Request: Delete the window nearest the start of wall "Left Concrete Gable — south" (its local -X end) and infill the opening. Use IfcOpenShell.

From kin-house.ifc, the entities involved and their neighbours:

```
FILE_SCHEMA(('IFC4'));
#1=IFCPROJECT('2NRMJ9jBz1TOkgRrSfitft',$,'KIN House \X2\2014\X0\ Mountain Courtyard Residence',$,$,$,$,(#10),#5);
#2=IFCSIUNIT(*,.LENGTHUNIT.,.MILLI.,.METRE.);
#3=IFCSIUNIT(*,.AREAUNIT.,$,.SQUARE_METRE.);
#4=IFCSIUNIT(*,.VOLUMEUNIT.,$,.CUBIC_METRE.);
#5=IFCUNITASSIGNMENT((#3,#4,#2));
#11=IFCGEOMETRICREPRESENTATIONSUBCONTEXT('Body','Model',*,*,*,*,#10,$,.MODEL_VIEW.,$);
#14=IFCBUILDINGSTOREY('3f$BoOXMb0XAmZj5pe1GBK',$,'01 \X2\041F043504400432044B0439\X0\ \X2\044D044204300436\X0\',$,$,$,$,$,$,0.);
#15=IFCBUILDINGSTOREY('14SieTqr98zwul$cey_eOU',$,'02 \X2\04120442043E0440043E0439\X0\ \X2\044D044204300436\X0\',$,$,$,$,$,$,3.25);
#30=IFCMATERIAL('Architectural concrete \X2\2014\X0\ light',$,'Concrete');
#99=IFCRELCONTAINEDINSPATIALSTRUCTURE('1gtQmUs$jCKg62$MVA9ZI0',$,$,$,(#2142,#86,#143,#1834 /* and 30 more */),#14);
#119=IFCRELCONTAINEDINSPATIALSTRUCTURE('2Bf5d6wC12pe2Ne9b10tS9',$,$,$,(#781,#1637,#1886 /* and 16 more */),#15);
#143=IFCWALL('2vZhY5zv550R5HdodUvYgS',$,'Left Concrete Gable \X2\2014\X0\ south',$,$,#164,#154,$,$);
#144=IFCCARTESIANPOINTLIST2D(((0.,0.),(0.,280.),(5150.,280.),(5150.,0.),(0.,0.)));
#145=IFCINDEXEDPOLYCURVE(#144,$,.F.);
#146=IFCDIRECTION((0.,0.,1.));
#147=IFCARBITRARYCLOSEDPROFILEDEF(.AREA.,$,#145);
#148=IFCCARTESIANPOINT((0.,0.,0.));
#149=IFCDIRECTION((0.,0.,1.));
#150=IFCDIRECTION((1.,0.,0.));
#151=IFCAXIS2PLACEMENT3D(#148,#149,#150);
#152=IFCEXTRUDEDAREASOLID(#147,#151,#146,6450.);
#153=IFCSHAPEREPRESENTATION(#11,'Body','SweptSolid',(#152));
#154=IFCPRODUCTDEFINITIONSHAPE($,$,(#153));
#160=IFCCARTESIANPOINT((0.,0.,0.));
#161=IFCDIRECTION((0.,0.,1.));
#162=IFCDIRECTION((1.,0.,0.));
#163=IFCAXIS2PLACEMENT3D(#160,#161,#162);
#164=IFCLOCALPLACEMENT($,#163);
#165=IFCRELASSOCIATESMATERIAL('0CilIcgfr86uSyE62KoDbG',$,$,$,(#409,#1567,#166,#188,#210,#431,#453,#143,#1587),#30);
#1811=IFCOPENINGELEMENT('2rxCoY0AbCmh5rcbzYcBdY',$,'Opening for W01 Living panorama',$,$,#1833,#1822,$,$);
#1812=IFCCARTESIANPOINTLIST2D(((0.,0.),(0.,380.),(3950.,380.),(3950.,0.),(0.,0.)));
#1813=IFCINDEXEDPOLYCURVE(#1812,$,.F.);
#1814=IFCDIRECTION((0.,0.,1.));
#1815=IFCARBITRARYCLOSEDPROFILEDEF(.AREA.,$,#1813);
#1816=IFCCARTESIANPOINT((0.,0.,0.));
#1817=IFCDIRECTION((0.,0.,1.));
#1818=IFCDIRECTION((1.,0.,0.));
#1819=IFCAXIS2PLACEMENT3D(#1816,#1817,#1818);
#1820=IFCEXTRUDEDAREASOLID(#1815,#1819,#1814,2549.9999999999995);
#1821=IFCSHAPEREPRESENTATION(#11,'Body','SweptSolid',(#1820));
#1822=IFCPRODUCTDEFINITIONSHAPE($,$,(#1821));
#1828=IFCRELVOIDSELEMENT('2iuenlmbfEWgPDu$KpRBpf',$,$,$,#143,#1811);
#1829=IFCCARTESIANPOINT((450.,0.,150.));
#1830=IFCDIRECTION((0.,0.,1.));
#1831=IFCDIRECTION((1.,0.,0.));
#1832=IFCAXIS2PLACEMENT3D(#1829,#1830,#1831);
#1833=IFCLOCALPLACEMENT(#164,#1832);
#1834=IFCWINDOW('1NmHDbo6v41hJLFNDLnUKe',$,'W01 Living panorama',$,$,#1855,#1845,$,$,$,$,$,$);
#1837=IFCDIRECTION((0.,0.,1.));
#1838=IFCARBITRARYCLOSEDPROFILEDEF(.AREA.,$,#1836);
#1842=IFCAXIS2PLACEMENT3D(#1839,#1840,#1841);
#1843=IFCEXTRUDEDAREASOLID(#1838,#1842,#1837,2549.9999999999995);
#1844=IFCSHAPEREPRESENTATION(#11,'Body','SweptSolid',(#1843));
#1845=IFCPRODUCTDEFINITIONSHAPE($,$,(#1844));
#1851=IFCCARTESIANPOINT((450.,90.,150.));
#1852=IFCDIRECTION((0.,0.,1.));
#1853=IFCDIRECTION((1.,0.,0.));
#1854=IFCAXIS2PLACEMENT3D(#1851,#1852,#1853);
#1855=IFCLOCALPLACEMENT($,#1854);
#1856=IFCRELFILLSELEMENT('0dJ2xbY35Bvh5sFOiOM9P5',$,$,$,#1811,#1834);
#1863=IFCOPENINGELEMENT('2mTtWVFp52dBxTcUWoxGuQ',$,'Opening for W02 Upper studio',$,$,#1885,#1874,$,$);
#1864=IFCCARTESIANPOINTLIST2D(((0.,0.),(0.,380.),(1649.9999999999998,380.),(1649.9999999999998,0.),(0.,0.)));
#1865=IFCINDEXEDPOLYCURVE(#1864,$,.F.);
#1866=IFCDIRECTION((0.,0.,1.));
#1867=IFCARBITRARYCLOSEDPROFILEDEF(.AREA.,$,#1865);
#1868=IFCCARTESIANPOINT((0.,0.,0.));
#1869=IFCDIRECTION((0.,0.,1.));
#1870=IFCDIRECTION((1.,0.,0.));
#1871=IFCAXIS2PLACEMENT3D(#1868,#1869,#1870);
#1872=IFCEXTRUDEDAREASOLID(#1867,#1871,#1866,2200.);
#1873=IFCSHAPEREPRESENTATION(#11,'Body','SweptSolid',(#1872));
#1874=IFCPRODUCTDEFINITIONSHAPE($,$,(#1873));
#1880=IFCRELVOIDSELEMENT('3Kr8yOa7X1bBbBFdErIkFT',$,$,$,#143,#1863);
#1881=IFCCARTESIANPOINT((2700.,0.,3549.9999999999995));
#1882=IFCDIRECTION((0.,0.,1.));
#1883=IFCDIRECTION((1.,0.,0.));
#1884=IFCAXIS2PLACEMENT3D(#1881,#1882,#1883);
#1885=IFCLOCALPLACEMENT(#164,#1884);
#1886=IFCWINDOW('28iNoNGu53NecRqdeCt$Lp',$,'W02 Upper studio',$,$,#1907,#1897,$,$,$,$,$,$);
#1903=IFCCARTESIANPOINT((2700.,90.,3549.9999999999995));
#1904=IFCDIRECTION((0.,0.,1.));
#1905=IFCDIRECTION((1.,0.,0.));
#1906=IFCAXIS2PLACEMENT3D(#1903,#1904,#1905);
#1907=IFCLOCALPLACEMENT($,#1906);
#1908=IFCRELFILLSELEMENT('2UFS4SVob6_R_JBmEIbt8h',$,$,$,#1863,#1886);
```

```python
import ifcopenshell
import ifcopenshell.api.feature
import ifcopenshell.api.root
import ifcopenshell.geom
import ifcopenshell.util.shape

model = ifcopenshell.open("kin-house.ifc")
settings = ifcopenshell.geom.settings()


def volume(element):
    """Net volume in cubic metres, openings subtracted."""
    shape = ifcopenshell.geom.create_shape(settings, element)
    return ifcopenshell.util.shape.get_volume(shape.geometry)


window = model.by_id(1834)
opening = window.FillsVoids[0].RelatingOpeningElement
wall = opening.VoidsElements[0].RelatingBuildingElement
before = volume(wall)

ifcopenshell.api.root.remove_product(model, product=window)
ifcopenshell.api.feature.remove_feature(model, feature=opening)

after = volume(wall)

print(f"wall volume {before:.3f} -> {after:.3f} m3")

model.write("kin-house_rev.ifc")
```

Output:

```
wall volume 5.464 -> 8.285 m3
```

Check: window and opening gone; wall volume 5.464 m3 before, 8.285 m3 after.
